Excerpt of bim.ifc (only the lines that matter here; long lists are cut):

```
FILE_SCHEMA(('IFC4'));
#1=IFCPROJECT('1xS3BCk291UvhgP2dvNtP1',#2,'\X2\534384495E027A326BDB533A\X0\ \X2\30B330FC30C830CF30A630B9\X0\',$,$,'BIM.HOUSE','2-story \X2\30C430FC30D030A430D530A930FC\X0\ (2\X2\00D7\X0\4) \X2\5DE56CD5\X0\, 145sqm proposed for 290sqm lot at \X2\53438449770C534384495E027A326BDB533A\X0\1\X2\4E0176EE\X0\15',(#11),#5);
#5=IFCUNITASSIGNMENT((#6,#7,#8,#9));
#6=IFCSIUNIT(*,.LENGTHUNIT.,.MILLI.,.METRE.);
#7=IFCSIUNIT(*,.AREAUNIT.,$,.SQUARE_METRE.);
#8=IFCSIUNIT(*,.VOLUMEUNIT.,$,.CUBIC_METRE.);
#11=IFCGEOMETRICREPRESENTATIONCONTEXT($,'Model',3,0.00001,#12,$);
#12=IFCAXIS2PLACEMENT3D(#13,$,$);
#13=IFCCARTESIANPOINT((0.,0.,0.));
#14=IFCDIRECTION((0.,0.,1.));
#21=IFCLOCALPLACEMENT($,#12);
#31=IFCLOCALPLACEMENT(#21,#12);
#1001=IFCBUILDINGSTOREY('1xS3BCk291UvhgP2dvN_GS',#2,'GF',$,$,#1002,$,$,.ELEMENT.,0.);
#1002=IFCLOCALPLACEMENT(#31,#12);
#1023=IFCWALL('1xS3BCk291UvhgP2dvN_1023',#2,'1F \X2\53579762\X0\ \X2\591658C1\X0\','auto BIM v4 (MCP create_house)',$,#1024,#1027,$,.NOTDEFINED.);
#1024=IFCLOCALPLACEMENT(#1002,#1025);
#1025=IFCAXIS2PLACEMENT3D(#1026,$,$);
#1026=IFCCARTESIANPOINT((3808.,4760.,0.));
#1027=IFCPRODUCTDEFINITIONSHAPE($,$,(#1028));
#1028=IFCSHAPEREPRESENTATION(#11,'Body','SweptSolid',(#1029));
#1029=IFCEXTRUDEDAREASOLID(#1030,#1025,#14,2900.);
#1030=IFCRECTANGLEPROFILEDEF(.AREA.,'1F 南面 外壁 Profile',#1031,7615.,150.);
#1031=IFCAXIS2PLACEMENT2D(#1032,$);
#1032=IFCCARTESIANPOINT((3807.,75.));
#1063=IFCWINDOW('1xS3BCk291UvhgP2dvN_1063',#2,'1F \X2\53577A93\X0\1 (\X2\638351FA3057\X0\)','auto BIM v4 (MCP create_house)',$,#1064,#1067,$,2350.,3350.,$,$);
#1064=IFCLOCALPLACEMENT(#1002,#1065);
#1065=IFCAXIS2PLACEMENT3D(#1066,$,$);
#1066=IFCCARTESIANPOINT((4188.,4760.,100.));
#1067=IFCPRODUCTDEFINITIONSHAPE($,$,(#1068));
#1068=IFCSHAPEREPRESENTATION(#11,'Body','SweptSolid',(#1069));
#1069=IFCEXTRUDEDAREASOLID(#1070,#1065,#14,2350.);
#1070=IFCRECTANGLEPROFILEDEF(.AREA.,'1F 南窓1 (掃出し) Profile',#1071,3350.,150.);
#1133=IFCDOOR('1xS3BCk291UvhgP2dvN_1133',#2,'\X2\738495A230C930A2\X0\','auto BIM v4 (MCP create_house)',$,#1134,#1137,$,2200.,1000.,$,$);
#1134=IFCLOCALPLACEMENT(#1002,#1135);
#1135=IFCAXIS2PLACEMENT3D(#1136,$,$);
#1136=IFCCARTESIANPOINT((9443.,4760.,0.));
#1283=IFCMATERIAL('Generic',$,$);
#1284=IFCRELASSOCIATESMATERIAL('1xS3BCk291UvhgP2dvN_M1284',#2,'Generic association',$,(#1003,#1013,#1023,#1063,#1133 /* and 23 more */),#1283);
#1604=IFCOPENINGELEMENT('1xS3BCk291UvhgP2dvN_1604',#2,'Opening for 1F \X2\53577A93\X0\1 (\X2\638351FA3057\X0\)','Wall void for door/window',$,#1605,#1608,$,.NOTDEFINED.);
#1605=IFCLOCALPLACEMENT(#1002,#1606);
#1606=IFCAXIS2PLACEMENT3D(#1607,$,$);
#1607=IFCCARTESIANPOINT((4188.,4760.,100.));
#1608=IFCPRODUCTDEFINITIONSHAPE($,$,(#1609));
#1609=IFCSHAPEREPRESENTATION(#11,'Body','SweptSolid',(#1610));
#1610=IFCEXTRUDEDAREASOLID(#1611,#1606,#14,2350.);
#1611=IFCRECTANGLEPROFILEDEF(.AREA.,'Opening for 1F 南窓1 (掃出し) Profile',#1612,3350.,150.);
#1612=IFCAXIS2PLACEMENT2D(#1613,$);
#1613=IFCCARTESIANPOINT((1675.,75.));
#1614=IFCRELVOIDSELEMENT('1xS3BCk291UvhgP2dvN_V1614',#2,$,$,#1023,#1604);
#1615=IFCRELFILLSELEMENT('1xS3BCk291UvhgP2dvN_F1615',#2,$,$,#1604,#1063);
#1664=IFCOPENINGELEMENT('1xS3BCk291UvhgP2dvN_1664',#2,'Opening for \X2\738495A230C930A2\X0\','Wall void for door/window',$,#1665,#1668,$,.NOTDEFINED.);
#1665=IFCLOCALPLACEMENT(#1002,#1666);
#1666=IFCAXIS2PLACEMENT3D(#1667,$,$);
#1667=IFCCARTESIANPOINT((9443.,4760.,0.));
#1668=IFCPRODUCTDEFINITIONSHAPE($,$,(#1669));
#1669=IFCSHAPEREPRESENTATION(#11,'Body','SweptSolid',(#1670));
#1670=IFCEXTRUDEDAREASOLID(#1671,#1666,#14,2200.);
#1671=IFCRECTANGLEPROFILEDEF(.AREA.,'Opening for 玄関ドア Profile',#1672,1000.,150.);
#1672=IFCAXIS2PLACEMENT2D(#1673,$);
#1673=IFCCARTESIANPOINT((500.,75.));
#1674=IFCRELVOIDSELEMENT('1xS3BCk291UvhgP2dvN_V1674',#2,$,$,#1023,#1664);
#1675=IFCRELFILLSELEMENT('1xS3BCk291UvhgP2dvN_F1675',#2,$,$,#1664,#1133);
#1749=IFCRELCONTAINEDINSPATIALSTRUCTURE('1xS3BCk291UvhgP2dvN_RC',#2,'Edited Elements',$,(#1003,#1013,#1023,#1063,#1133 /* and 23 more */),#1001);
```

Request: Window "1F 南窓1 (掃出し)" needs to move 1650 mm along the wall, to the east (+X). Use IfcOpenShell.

```python
import ifcopenshell
import ifcopenshell.api.geometry
import ifcopenshell.util.placement

model = ifcopenshell.open("bim.ifc")

window = model.by_guid("1xS3BCk291UvhgP2dvN_1063")
opening = window.FillsVoids[0].RelatingOpeningElement
wall = opening.VoidsElements[0].RelatingBuildingElement

wall_matrix = ifcopenshell.util.placement.get_local_placement(wall.ObjectPlacement)
shift = wall_matrix[:3, 0] * 1650.0
before = ifcopenshell.util.placement.get_local_placement(window.ObjectPlacement)[:3, 3].copy()

# The window is not placed relative to its opening, so move both.
for product in (opening, window):
    matrix = ifcopenshell.util.placement.get_local_placement(product.ObjectPlacement)
    matrix[:3, 3] += shift
    ifcopenshell.api.geometry.edit_object_placement(model, product=product, matrix=matrix, is_si=False)

after = ifcopenshell.util.placement.get_local_placement(window.ObjectPlacement)[:3, 3]
print("window moved by", (after - before).round(3) + 0.0)

model.write("bim_updated.ifc")
```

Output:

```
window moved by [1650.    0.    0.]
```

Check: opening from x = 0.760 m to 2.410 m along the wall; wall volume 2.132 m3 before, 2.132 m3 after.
